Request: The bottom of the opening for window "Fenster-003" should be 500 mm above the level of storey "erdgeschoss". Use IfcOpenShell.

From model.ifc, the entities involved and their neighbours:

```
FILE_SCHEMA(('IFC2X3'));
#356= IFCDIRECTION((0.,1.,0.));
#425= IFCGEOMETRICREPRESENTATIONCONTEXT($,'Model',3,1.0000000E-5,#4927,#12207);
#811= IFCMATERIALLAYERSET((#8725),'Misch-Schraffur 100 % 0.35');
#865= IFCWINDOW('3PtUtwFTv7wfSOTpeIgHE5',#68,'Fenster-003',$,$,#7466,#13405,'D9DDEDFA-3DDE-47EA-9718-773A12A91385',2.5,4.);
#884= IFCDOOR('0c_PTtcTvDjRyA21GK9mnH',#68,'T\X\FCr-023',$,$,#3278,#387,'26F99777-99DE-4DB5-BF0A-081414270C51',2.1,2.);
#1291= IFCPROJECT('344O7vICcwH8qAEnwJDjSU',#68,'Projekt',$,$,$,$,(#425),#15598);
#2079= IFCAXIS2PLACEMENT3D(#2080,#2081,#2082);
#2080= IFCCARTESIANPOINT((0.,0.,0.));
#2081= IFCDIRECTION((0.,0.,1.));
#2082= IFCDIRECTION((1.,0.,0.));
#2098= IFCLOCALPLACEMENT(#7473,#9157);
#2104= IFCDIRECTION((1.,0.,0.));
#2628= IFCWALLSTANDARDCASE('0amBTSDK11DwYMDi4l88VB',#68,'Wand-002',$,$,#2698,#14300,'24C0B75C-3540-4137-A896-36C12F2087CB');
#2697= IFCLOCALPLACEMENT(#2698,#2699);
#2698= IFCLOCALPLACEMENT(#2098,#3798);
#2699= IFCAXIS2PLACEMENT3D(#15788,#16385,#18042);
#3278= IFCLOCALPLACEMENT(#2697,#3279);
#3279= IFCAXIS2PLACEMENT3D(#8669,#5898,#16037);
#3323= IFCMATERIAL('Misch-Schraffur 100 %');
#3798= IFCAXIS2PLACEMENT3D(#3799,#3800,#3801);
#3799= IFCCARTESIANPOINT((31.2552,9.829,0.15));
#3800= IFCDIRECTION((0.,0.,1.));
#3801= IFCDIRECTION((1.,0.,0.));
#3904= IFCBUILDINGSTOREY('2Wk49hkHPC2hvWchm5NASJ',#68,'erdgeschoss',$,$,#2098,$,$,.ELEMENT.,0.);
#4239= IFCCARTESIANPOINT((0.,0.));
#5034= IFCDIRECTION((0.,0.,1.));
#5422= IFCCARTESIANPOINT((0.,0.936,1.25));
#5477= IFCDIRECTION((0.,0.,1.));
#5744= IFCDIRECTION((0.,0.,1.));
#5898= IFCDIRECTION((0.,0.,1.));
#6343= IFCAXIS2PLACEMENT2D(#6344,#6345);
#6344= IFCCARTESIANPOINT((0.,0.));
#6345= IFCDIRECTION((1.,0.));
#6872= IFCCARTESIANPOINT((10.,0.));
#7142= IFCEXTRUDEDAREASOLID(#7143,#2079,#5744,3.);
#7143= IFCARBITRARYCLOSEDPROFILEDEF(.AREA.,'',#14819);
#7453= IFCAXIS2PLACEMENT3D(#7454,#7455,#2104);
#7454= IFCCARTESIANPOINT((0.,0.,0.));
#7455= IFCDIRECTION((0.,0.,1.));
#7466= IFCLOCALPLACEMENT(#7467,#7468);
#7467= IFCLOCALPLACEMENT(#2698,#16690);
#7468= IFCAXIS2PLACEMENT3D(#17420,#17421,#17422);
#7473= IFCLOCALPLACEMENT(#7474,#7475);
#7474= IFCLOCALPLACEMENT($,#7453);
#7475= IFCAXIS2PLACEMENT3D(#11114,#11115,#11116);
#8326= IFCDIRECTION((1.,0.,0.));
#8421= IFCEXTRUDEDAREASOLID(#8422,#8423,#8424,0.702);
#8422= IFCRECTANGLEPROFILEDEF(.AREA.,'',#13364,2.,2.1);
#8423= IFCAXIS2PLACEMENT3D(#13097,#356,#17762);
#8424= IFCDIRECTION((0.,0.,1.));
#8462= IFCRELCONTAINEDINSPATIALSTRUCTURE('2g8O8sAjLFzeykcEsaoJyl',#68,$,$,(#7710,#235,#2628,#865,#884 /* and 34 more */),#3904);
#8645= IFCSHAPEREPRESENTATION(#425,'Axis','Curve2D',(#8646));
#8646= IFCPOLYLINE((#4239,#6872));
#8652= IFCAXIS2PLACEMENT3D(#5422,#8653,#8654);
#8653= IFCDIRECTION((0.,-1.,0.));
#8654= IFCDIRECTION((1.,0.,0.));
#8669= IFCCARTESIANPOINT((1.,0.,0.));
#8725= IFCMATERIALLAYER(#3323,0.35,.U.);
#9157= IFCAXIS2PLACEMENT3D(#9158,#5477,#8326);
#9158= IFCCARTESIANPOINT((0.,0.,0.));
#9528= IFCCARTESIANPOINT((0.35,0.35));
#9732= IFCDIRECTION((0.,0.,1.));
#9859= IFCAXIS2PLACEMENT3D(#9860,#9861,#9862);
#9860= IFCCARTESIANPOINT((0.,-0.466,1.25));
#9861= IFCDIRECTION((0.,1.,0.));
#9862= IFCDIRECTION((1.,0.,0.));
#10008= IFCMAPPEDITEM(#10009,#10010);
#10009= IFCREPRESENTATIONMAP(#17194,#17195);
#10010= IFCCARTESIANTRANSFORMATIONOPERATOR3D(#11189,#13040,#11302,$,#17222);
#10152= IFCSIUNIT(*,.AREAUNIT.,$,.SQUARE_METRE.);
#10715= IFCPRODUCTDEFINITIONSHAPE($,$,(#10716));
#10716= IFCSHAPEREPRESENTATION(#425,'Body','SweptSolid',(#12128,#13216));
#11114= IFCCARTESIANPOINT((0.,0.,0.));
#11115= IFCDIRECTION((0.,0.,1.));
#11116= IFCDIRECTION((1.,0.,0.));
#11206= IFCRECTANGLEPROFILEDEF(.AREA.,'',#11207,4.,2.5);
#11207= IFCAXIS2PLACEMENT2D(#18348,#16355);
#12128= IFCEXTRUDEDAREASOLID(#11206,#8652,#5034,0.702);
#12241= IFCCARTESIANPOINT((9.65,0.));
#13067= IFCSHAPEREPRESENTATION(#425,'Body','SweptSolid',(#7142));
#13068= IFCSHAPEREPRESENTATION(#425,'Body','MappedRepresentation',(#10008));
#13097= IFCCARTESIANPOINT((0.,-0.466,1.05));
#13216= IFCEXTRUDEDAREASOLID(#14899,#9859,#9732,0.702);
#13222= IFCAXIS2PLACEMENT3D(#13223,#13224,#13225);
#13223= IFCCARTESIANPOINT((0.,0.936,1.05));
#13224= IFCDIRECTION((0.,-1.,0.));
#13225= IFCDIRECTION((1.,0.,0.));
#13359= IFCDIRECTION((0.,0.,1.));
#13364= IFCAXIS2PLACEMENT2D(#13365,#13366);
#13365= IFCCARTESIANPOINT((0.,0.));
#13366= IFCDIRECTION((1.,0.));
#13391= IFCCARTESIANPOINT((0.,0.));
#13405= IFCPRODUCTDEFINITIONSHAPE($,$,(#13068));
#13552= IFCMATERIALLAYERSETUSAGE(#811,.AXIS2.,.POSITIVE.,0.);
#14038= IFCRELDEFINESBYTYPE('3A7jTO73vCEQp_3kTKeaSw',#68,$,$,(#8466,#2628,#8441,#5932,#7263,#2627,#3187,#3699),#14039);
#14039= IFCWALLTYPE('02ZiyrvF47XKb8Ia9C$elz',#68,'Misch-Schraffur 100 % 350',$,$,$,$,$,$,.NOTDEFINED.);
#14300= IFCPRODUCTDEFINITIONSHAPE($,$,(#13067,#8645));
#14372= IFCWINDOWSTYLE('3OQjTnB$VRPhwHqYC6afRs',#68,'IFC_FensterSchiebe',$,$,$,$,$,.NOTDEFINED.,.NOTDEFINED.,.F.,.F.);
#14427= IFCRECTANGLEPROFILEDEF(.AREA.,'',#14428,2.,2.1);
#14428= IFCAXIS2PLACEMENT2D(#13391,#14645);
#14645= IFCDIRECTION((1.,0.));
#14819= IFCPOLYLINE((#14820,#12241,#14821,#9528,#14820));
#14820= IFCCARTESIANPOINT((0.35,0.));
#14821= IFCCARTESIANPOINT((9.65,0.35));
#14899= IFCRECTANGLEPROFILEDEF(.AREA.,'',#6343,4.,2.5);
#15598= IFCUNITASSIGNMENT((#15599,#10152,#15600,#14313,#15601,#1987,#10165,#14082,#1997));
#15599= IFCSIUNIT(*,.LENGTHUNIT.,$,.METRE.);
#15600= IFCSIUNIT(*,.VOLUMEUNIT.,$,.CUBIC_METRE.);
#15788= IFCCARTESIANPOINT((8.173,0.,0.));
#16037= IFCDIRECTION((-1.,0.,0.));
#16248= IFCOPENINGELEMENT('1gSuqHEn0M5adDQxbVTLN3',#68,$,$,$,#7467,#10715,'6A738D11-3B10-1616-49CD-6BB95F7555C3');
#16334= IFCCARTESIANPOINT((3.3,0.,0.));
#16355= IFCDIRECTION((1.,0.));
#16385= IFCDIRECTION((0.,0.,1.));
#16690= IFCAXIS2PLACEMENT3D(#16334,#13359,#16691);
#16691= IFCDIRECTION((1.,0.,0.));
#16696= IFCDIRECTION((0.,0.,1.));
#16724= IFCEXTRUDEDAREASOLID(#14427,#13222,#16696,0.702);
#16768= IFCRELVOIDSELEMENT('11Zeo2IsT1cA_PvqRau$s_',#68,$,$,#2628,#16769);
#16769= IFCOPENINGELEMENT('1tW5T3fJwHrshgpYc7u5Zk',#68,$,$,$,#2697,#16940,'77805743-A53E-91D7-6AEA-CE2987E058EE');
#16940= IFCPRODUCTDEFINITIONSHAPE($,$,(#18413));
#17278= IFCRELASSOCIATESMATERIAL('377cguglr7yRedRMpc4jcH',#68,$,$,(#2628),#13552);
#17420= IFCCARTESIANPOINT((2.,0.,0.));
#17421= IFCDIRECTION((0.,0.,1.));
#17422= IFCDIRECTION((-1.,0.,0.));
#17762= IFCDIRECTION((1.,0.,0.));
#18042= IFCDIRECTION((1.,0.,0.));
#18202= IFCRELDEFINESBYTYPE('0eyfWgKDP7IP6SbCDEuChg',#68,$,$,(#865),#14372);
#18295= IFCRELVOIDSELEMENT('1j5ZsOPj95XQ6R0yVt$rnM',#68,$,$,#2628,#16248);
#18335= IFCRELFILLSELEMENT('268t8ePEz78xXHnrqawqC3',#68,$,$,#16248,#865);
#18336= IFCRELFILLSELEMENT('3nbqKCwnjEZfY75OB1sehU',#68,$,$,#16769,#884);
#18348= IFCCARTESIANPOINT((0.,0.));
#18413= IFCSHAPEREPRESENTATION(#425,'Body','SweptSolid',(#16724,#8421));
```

```python
import numpy as np
import ifcopenshell
import ifcopenshell.api.geometry
import ifcopenshell.geom
import ifcopenshell.util.element
import ifcopenshell.util.placement
import ifcopenshell.util.shape
import ifcopenshell.util.unit

model = ifcopenshell.open("model.ifc")
unit_scale = ifcopenshell.util.unit.calculate_unit_scale(model)

window = model.by_guid("3PtUtwFTv7wfSOTpeIgHE5")
opening = window.FillsVoids[0].RelatingOpeningElement
storey = ifcopenshell.util.element.get_container(window, ifc_class="IfcBuildingStorey")
level = ifcopenshell.util.placement.get_local_placement(storey.ObjectPlacement)[2, 3]

# The opening's origin need not be at the sill, so measure its lowest point.
shape = ifcopenshell.geom.create_shape(ifcopenshell.geom.settings(), opening)
bottom = ifcopenshell.util.shape.get_shape_bottom_elevation(shape, shape.geometry) / unit_scale
dz = level + 0.5 / unit_scale - bottom

shift = np.array([0.0, 0.0, dz])
# The window is placed relative to its opening, so it follows when the opening moves.
matrix = ifcopenshell.util.placement.get_local_placement(opening.ObjectPlacement)
matrix[:3, 3] += shift
ifcopenshell.api.geometry.edit_object_placement(
    model, product=opening, matrix=matrix, is_si=False, should_transform_children=True
)

print(f"moved by {dz * unit_scale:+.3f} m")

model.write("model_rev.ifc")
```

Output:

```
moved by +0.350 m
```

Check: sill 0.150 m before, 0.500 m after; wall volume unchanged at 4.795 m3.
